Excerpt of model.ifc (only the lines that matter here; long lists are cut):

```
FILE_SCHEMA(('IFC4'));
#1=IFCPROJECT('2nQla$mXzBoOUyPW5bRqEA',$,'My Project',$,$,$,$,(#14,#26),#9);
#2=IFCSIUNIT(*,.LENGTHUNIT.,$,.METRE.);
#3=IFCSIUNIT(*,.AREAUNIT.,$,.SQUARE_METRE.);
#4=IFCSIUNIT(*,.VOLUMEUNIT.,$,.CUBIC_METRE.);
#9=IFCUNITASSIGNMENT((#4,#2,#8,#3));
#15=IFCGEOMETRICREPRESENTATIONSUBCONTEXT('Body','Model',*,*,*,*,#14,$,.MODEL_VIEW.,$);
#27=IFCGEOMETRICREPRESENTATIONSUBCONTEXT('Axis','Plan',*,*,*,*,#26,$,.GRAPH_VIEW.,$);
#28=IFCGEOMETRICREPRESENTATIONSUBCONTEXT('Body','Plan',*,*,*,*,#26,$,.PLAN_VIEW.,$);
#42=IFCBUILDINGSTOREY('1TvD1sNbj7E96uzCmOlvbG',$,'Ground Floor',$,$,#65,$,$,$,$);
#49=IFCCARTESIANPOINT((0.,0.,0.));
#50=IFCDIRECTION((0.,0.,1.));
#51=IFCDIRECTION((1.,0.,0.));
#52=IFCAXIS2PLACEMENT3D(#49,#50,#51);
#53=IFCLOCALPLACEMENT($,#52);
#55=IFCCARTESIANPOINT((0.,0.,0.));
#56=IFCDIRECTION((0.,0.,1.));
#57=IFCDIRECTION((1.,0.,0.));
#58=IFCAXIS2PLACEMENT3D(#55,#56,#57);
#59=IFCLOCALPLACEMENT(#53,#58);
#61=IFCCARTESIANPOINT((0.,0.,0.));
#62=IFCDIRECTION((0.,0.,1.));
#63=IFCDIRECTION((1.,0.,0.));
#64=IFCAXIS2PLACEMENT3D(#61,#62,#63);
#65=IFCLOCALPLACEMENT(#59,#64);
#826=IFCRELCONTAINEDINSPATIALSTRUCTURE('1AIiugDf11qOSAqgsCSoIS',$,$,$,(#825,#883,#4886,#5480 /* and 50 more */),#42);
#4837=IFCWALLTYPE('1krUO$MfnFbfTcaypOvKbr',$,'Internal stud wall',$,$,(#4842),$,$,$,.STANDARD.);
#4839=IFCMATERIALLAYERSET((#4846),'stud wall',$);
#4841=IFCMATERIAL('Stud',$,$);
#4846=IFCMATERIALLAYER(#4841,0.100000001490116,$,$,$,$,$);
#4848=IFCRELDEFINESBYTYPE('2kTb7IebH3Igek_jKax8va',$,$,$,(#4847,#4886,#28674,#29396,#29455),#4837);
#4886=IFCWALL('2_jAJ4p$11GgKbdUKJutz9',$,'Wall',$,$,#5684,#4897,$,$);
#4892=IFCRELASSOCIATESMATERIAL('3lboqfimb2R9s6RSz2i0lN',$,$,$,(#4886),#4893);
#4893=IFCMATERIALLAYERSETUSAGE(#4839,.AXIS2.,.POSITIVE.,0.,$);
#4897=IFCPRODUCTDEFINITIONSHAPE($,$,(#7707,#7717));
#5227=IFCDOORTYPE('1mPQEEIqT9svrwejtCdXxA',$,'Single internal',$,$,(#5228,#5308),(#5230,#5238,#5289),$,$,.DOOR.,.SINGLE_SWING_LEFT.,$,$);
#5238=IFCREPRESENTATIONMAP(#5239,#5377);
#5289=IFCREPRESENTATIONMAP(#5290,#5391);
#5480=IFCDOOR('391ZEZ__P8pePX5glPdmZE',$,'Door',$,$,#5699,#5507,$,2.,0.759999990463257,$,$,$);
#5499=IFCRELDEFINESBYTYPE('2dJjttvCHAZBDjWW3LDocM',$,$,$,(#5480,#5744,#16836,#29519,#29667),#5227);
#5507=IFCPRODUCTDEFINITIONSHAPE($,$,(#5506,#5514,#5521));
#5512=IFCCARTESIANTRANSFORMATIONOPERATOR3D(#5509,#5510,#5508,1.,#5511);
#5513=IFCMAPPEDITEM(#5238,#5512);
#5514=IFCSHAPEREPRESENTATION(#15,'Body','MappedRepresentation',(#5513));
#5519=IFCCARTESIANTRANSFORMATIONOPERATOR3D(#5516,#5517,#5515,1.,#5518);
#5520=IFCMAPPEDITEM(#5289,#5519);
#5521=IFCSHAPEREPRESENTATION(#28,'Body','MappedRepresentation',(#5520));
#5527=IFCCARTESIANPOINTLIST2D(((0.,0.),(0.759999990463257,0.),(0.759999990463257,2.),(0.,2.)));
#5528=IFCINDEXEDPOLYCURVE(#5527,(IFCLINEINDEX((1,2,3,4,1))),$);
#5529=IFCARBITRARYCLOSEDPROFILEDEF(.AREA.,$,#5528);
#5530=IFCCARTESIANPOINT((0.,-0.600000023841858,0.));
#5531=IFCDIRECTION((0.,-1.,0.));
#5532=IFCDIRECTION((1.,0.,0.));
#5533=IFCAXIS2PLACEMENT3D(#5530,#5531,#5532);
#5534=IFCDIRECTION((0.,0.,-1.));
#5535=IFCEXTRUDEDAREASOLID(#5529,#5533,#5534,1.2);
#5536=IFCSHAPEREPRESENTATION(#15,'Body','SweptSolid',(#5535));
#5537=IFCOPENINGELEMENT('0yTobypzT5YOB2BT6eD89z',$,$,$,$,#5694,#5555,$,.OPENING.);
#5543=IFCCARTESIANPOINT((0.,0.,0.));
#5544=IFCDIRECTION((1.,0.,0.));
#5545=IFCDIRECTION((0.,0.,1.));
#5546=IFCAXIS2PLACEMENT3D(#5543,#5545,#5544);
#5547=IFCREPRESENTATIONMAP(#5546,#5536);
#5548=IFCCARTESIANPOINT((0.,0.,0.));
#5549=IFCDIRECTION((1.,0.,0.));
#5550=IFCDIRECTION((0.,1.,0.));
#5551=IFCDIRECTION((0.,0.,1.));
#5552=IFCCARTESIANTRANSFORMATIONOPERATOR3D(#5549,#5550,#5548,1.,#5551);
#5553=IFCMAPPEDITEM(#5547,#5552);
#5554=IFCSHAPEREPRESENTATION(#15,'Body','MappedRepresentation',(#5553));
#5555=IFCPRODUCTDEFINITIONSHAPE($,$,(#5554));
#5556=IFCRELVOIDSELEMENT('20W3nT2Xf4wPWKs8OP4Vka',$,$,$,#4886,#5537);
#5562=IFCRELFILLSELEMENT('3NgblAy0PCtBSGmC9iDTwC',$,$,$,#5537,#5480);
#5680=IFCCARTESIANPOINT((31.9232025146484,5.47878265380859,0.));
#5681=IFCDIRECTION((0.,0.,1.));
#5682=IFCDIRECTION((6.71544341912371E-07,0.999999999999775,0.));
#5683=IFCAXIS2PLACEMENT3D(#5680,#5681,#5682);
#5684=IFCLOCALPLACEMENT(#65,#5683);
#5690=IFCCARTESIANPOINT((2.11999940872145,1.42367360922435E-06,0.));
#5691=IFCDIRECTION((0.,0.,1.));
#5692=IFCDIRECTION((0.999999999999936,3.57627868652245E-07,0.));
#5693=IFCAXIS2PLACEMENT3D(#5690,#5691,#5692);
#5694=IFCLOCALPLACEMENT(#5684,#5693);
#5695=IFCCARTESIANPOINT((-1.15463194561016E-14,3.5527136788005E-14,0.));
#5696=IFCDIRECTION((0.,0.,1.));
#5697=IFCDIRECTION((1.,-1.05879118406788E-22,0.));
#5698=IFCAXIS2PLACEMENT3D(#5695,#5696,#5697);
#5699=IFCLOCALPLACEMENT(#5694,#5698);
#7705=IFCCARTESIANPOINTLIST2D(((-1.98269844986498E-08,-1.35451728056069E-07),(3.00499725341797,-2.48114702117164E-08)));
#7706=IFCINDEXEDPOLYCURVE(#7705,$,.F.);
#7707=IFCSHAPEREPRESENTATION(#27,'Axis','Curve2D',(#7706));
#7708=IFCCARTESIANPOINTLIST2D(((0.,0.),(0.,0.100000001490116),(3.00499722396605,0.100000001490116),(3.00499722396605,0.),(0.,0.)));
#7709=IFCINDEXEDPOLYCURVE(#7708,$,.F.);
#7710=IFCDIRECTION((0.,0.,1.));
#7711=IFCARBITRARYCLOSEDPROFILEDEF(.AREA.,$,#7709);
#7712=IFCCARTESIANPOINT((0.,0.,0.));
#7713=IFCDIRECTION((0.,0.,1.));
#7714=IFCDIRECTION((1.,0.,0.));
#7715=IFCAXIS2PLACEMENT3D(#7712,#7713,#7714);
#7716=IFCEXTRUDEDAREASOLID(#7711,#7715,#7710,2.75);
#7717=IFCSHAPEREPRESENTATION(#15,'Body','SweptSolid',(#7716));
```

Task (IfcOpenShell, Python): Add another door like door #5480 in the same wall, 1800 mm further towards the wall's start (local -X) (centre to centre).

```python
import ifcopenshell
import ifcopenshell.api.feature
import ifcopenshell.api.geometry
import ifcopenshell.api.root
import ifcopenshell.geom
import ifcopenshell.util.element
import ifcopenshell.util.placement
import ifcopenshell.util.shape
import ifcopenshell.util.unit

model = ifcopenshell.open("model.ifc")
unit_scale = ifcopenshell.util.unit.calculate_unit_scale(model)
settings = ifcopenshell.geom.settings()


def volume(element):
    """Net volume in cubic metres, openings subtracted."""
    shape = ifcopenshell.geom.create_shape(settings, element)
    return ifcopenshell.util.shape.get_volume(shape.geometry)


door = model.by_id(5480)
opening = door.FillsVoids[0].RelatingOpeningElement
wall = opening.VoidsElements[0].RelatingBuildingElement
before = volume(wall)
shift = ifcopenshell.util.placement.get_local_placement(wall.ObjectPlacement)[:3, 0] * -1.8 / unit_scale

# copy_class copies the void relationship, type, container and properties, but no geometry.
new_opening = ifcopenshell.api.root.copy_class(model, product=opening)
new_opening.Representation = ifcopenshell.util.element.copy_deep(
    model, opening.Representation, exclude=["IfcGeometricRepresentationContext", "IfcRepresentationMap"]
)
new_door = ifcopenshell.api.root.copy_class(model, product=door)
new_door.Representation = ifcopenshell.util.element.copy_deep(
    model, door.Representation, exclude=["IfcGeometricRepresentationContext", "IfcRepresentationMap"]
)
ifcopenshell.api.feature.add_filling(model, opening=new_opening, element=new_door)

for old, new in ((opening, new_opening), (door, new_door)):
    matrix = ifcopenshell.util.placement.get_local_placement(old.ObjectPlacement)
    matrix[:3, 3] += shift
    ifcopenshell.api.geometry.edit_object_placement(model, product=new, matrix=matrix, is_si=False)

after = volume(wall)

print(f"wall volume {before:.3f} -> {after:.3f} m3")

model.write("model_updated.ifc")
```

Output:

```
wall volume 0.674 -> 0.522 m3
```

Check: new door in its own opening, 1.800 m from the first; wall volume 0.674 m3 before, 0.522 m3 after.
